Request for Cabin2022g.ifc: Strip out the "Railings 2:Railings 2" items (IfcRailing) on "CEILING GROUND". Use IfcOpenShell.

First a look at what the model holds.

```python
import ifcopenshell
import ifcopenshell.util.element

model = ifcopenshell.open("Cabin2022g.ifc")
print(model.schema)
storey = next(s for s in model.by_type("IfcBuildingStorey") if s.Name == "CEILING GROUND")
railings = [e for e in ifcopenshell.util.element.get_decomposition(storey) if e.is_a("IfcRailing")]
seen = {}
for e in railings:
    element_type = ifcopenshell.util.element.get_type(e)
    name = element_type.Name if element_type not in (None, e) else None
    seen[name] = seen.get(name, 0) + 1
for name, count in sorted(seen.items(), key=str):
    print(count, "x", name)
```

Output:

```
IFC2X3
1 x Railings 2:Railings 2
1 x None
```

```python
import ifcopenshell
import ifcopenshell.api.root
import ifcopenshell.util.element

model = ifcopenshell.open("Cabin2022g.ifc")

storey = next(s for s in model.by_type("IfcBuildingStorey") if s.Name == "CEILING GROUND")
railings = [e for e in ifcopenshell.util.element.get_decomposition(storey) if e.is_a("IfcRailing")]
targets = [e for e in railings if (t := ifcopenshell.util.element.get_type(e)) not in (None, e) and t.Name == "Railings 2:Railings 2"]

for e in targets:
    ifcopenshell.api.root.remove_product(model, product=e)
print(len(targets), "removed")

model.write("Cabin2022g-out.ifc")
```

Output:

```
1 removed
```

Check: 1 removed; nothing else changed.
